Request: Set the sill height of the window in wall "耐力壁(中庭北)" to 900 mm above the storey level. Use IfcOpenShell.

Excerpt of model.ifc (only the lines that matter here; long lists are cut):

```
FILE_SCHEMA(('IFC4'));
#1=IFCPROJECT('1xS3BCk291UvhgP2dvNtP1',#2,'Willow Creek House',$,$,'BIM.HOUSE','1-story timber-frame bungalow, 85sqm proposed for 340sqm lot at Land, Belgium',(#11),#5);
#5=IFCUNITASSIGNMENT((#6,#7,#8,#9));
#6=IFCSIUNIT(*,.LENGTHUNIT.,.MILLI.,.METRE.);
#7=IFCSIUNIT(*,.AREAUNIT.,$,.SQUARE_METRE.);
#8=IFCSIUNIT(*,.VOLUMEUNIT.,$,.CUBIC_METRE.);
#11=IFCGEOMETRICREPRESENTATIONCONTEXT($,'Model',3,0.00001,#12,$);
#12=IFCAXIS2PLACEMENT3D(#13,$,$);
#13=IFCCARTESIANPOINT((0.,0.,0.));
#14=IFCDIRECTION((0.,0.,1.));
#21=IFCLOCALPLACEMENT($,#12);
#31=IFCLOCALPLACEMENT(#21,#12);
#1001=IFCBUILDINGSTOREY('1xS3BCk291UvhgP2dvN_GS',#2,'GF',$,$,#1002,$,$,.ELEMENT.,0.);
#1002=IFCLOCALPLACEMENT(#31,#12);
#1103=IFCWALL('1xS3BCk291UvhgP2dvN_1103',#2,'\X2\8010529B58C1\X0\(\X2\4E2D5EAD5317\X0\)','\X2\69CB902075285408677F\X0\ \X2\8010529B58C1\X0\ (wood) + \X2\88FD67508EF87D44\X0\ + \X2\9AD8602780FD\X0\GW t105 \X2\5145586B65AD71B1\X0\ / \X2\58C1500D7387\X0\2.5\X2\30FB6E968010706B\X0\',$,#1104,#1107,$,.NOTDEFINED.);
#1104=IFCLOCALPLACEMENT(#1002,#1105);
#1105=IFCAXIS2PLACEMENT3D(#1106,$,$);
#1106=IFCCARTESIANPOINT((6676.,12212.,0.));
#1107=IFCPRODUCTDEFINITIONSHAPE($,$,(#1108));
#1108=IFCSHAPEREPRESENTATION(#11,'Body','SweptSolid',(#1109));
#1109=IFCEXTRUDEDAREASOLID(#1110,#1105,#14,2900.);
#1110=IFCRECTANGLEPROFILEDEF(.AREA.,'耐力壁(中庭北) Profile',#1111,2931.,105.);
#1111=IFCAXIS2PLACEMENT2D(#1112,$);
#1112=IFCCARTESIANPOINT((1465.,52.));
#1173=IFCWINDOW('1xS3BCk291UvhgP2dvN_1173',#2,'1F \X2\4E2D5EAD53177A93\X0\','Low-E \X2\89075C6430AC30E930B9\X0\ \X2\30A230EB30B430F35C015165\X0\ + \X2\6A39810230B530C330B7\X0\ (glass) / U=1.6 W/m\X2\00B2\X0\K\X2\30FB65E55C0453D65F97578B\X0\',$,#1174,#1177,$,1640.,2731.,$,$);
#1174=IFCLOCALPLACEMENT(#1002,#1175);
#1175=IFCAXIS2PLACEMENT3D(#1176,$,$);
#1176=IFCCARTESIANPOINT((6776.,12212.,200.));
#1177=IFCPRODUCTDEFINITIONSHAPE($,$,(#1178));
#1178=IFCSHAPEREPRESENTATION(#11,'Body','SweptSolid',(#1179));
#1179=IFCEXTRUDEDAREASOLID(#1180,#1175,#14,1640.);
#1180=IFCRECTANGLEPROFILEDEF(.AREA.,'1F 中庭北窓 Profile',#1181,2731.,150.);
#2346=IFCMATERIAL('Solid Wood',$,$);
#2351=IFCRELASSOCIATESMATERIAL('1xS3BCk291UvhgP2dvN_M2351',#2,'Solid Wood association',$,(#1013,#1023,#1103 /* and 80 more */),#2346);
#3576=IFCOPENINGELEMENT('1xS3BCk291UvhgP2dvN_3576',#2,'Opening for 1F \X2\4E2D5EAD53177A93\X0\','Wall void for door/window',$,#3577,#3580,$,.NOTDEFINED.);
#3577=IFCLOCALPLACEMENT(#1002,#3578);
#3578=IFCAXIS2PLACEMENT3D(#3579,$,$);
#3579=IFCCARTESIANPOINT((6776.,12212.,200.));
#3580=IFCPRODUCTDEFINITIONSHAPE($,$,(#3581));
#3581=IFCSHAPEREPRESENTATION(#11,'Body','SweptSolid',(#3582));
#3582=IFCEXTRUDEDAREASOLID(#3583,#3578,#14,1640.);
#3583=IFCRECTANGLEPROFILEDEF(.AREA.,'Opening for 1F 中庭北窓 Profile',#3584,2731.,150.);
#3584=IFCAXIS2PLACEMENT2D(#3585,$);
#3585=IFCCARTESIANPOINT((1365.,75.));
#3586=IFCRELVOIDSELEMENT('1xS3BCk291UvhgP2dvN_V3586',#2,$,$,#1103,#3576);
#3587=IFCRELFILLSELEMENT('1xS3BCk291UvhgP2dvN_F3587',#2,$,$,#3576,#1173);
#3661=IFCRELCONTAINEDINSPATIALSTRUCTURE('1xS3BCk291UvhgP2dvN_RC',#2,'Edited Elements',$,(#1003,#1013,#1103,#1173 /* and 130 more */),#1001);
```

```python
import numpy as np
import ifcopenshell
import ifcopenshell.api.geometry
import ifcopenshell.geom
import ifcopenshell.util.element
import ifcopenshell.util.placement
import ifcopenshell.util.shape
import ifcopenshell.util.unit

model = ifcopenshell.open("model.ifc")
unit_scale = ifcopenshell.util.unit.calculate_unit_scale(model)

window = model.by_id(1173)
opening = window.FillsVoids[0].RelatingOpeningElement
storey = ifcopenshell.util.element.get_container(window, ifc_class="IfcBuildingStorey")
level = ifcopenshell.util.placement.get_local_placement(storey.ObjectPlacement)[2, 3]

# The opening's origin need not be at the sill, so measure its lowest point.
shape = ifcopenshell.geom.create_shape(ifcopenshell.geom.settings(), opening)
bottom = ifcopenshell.util.shape.get_shape_bottom_elevation(shape, shape.geometry) / unit_scale
dz = level + 0.9 / unit_scale - bottom

shift = np.array([0.0, 0.0, dz])
# The window is not placed relative to its opening, so move both.
for product in (opening, window):
    matrix = ifcopenshell.util.placement.get_local_placement(product.ObjectPlacement)
    matrix[:3, 3] += shift
    ifcopenshell.api.geometry.edit_object_placement(model, product=product, matrix=matrix, is_si=False)

print(f"moved by {dz * unit_scale:+.3f} m")

model.write("model_edited.ifc")
```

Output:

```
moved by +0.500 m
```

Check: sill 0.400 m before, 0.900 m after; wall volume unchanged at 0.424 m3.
